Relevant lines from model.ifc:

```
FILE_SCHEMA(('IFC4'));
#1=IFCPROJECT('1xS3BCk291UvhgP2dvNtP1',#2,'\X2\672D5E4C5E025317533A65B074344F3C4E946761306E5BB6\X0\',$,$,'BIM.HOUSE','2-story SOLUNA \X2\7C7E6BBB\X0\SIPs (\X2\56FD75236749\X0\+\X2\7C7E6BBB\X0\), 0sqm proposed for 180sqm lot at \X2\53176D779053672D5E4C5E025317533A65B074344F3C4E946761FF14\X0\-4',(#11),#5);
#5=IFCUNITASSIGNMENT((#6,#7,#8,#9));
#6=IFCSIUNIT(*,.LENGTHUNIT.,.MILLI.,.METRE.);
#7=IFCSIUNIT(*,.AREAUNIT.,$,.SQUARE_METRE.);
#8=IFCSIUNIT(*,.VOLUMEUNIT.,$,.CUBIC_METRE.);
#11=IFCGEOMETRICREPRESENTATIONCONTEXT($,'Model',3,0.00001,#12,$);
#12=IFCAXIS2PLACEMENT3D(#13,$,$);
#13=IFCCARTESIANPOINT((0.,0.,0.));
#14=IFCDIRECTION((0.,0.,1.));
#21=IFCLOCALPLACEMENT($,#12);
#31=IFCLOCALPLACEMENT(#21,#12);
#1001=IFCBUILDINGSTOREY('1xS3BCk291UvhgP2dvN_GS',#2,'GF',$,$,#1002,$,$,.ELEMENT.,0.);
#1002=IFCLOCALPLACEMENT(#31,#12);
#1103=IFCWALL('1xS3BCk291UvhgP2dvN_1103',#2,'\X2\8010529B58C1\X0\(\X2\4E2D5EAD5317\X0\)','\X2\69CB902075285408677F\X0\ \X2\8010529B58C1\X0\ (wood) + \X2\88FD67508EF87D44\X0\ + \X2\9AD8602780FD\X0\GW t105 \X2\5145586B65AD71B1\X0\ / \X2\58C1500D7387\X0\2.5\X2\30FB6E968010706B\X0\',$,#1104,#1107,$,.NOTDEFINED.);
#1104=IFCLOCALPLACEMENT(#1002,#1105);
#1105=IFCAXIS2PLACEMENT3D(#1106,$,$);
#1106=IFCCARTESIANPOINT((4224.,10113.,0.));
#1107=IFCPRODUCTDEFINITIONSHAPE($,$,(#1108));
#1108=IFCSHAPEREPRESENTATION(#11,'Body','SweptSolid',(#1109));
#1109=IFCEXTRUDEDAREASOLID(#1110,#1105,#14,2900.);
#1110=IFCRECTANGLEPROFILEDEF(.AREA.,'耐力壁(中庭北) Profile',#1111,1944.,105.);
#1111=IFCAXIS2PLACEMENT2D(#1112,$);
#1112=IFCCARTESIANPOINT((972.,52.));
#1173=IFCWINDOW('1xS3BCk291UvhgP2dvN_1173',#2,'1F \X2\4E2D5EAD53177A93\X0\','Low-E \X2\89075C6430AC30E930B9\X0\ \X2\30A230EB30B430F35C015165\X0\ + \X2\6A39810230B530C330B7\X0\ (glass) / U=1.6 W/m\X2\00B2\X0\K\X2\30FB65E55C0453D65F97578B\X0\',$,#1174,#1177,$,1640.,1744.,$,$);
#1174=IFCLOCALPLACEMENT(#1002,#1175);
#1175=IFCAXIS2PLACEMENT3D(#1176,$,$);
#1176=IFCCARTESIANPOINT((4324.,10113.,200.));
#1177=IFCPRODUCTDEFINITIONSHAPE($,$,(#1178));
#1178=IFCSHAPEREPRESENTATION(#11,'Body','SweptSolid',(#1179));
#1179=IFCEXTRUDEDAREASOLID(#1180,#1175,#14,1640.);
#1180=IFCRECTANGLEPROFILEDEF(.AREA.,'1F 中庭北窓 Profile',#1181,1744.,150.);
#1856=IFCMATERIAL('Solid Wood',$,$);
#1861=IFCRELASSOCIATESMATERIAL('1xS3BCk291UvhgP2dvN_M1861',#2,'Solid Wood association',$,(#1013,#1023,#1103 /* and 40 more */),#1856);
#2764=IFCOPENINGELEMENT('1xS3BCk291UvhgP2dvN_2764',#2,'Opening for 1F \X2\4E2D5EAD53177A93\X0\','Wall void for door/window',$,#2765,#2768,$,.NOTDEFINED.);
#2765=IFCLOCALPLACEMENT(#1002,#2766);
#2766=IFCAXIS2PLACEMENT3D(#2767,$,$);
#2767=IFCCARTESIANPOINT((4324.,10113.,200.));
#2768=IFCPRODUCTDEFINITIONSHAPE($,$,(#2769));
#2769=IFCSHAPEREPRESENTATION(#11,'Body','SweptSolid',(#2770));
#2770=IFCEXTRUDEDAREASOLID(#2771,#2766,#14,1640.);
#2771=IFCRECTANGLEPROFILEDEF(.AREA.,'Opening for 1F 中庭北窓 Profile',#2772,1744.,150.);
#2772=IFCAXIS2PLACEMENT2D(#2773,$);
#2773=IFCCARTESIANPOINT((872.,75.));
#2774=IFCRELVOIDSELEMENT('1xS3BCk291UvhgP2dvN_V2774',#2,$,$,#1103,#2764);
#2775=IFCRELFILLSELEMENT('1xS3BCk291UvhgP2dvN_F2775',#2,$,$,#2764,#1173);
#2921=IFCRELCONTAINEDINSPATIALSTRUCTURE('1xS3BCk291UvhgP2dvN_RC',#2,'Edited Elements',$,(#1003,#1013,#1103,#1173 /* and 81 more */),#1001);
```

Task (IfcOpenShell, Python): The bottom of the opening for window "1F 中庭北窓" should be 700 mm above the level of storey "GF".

```python
import numpy as np
import ifcopenshell
import ifcopenshell.api.geometry
import ifcopenshell.geom
import ifcopenshell.util.element
import ifcopenshell.util.placement
import ifcopenshell.util.shape
import ifcopenshell.util.unit

model = ifcopenshell.open("model.ifc")
unit_scale = ifcopenshell.util.unit.calculate_unit_scale(model)

window = model.by_id(1173)
opening = window.FillsVoids[0].RelatingOpeningElement
storey = ifcopenshell.util.element.get_container(window, ifc_class="IfcBuildingStorey")
level = ifcopenshell.util.placement.get_local_placement(storey.ObjectPlacement)[2, 3]

# The opening's origin need not be at the sill, so measure its lowest point.
shape = ifcopenshell.geom.create_shape(ifcopenshell.geom.settings(), opening)
bottom = ifcopenshell.util.shape.get_shape_bottom_elevation(shape, shape.geometry) / unit_scale
dz = level + 0.7 / unit_scale - bottom

shift = np.array([0.0, 0.0, dz])
# The window is not placed relative to its opening, so move both.
for product in (opening, window):
    matrix = ifcopenshell.util.placement.get_local_placement(product.ObjectPlacement)
    matrix[:3, 3] += shift
    ifcopenshell.api.geometry.edit_object_placement(model, product=product, matrix=matrix, is_si=False)

print(f"moved by {dz * unit_scale:+.3f} m")

model.write("model_edited.ifc")
```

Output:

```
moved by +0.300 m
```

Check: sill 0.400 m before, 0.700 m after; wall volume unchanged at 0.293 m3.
